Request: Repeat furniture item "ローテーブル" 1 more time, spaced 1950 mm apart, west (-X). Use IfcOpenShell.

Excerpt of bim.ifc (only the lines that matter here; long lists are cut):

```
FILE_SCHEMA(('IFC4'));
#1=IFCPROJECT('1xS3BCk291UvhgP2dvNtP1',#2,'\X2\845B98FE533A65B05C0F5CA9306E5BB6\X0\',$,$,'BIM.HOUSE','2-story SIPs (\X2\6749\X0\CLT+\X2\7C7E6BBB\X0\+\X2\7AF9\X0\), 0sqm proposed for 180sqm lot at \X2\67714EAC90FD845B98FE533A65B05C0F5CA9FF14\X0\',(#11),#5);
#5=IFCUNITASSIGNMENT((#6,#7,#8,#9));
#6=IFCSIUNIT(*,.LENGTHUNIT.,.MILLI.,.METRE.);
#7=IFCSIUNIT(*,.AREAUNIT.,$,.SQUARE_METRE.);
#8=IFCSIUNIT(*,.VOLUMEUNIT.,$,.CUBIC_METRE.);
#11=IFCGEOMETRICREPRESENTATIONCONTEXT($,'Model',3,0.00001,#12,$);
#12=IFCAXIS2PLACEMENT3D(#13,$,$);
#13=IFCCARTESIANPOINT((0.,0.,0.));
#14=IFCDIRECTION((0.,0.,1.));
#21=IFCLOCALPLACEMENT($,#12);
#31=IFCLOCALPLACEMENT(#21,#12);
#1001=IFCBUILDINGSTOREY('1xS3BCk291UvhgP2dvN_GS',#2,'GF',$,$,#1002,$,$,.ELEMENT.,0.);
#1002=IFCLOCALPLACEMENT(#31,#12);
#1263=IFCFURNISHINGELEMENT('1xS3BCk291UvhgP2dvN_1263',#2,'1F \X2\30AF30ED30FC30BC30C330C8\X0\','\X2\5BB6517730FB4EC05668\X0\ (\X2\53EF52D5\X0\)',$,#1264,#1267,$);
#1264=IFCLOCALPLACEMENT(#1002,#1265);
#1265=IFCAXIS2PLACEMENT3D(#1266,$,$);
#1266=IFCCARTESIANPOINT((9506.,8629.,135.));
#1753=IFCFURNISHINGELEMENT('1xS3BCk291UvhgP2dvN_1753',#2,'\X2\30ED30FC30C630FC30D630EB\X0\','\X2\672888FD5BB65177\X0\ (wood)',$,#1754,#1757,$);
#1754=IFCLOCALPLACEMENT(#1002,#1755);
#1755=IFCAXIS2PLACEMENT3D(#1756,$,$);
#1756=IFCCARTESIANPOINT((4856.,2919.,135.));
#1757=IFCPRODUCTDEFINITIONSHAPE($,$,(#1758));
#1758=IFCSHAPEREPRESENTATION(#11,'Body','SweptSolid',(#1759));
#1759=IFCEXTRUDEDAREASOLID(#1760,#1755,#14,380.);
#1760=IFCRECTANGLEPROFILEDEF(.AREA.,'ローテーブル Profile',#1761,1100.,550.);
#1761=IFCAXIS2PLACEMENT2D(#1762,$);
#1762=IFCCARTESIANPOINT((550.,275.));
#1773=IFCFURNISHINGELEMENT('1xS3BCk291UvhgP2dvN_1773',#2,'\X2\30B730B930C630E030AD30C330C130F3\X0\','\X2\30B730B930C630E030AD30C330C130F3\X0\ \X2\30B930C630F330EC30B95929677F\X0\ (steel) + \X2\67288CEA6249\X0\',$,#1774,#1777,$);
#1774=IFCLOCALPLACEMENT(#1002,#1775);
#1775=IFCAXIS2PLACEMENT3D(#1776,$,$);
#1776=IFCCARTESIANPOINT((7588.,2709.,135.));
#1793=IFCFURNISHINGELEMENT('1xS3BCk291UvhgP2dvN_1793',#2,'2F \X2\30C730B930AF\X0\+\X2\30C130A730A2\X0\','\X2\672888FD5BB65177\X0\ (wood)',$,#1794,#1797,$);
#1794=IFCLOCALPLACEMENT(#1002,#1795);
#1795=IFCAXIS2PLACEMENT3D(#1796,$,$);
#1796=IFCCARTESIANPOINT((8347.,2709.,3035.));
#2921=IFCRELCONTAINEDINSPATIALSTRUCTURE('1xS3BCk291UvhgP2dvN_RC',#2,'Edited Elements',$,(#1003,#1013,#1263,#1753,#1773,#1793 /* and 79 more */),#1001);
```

```python
import numpy as np
import ifcopenshell
import ifcopenshell.api.geometry
import ifcopenshell.api.root
import ifcopenshell.util.element
import ifcopenshell.util.placement

model = ifcopenshell.open("bim.ifc")


def reuse_history(source, copy):
    """copy_class also copies each property set's owner history, people and application; keep the originals."""
    for rel in copy.IsDefinedBy:
        if rel.is_a("IfcRelDefinesByProperties") and (history := rel.RelatingPropertyDefinition.OwnerHistory):
            rel.RelatingPropertyDefinition.OwnerHistory = source.OwnerHistory
            ifcopenshell.util.element.remove_deep2(model, history)


source = model.by_guid("1xS3BCk291UvhgP2dvN_1753")
base = ifcopenshell.util.placement.get_local_placement(source.ObjectPlacement)
step = np.array([-1.0, 0.0, 0.0]) * 1950.0

for i in range(1, 2):
    copy = ifcopenshell.api.root.copy_class(model, product=source)
    copy.Representation = ifcopenshell.util.element.copy_deep(
        model, source.Representation, exclude=["IfcGeometricRepresentationContext", "IfcRepresentationMap"]
    )
    reuse_history(source, copy)
    matrix = base.copy()
    matrix[:3, 3] += i * step
    print("added at", matrix[:3, 3].round(3) + 0.0)
    ifcopenshell.api.geometry.edit_object_placement(model, product=copy, matrix=matrix, is_si=False)

model.write("bim_edited.ifc")
```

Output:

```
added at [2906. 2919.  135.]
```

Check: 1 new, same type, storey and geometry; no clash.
